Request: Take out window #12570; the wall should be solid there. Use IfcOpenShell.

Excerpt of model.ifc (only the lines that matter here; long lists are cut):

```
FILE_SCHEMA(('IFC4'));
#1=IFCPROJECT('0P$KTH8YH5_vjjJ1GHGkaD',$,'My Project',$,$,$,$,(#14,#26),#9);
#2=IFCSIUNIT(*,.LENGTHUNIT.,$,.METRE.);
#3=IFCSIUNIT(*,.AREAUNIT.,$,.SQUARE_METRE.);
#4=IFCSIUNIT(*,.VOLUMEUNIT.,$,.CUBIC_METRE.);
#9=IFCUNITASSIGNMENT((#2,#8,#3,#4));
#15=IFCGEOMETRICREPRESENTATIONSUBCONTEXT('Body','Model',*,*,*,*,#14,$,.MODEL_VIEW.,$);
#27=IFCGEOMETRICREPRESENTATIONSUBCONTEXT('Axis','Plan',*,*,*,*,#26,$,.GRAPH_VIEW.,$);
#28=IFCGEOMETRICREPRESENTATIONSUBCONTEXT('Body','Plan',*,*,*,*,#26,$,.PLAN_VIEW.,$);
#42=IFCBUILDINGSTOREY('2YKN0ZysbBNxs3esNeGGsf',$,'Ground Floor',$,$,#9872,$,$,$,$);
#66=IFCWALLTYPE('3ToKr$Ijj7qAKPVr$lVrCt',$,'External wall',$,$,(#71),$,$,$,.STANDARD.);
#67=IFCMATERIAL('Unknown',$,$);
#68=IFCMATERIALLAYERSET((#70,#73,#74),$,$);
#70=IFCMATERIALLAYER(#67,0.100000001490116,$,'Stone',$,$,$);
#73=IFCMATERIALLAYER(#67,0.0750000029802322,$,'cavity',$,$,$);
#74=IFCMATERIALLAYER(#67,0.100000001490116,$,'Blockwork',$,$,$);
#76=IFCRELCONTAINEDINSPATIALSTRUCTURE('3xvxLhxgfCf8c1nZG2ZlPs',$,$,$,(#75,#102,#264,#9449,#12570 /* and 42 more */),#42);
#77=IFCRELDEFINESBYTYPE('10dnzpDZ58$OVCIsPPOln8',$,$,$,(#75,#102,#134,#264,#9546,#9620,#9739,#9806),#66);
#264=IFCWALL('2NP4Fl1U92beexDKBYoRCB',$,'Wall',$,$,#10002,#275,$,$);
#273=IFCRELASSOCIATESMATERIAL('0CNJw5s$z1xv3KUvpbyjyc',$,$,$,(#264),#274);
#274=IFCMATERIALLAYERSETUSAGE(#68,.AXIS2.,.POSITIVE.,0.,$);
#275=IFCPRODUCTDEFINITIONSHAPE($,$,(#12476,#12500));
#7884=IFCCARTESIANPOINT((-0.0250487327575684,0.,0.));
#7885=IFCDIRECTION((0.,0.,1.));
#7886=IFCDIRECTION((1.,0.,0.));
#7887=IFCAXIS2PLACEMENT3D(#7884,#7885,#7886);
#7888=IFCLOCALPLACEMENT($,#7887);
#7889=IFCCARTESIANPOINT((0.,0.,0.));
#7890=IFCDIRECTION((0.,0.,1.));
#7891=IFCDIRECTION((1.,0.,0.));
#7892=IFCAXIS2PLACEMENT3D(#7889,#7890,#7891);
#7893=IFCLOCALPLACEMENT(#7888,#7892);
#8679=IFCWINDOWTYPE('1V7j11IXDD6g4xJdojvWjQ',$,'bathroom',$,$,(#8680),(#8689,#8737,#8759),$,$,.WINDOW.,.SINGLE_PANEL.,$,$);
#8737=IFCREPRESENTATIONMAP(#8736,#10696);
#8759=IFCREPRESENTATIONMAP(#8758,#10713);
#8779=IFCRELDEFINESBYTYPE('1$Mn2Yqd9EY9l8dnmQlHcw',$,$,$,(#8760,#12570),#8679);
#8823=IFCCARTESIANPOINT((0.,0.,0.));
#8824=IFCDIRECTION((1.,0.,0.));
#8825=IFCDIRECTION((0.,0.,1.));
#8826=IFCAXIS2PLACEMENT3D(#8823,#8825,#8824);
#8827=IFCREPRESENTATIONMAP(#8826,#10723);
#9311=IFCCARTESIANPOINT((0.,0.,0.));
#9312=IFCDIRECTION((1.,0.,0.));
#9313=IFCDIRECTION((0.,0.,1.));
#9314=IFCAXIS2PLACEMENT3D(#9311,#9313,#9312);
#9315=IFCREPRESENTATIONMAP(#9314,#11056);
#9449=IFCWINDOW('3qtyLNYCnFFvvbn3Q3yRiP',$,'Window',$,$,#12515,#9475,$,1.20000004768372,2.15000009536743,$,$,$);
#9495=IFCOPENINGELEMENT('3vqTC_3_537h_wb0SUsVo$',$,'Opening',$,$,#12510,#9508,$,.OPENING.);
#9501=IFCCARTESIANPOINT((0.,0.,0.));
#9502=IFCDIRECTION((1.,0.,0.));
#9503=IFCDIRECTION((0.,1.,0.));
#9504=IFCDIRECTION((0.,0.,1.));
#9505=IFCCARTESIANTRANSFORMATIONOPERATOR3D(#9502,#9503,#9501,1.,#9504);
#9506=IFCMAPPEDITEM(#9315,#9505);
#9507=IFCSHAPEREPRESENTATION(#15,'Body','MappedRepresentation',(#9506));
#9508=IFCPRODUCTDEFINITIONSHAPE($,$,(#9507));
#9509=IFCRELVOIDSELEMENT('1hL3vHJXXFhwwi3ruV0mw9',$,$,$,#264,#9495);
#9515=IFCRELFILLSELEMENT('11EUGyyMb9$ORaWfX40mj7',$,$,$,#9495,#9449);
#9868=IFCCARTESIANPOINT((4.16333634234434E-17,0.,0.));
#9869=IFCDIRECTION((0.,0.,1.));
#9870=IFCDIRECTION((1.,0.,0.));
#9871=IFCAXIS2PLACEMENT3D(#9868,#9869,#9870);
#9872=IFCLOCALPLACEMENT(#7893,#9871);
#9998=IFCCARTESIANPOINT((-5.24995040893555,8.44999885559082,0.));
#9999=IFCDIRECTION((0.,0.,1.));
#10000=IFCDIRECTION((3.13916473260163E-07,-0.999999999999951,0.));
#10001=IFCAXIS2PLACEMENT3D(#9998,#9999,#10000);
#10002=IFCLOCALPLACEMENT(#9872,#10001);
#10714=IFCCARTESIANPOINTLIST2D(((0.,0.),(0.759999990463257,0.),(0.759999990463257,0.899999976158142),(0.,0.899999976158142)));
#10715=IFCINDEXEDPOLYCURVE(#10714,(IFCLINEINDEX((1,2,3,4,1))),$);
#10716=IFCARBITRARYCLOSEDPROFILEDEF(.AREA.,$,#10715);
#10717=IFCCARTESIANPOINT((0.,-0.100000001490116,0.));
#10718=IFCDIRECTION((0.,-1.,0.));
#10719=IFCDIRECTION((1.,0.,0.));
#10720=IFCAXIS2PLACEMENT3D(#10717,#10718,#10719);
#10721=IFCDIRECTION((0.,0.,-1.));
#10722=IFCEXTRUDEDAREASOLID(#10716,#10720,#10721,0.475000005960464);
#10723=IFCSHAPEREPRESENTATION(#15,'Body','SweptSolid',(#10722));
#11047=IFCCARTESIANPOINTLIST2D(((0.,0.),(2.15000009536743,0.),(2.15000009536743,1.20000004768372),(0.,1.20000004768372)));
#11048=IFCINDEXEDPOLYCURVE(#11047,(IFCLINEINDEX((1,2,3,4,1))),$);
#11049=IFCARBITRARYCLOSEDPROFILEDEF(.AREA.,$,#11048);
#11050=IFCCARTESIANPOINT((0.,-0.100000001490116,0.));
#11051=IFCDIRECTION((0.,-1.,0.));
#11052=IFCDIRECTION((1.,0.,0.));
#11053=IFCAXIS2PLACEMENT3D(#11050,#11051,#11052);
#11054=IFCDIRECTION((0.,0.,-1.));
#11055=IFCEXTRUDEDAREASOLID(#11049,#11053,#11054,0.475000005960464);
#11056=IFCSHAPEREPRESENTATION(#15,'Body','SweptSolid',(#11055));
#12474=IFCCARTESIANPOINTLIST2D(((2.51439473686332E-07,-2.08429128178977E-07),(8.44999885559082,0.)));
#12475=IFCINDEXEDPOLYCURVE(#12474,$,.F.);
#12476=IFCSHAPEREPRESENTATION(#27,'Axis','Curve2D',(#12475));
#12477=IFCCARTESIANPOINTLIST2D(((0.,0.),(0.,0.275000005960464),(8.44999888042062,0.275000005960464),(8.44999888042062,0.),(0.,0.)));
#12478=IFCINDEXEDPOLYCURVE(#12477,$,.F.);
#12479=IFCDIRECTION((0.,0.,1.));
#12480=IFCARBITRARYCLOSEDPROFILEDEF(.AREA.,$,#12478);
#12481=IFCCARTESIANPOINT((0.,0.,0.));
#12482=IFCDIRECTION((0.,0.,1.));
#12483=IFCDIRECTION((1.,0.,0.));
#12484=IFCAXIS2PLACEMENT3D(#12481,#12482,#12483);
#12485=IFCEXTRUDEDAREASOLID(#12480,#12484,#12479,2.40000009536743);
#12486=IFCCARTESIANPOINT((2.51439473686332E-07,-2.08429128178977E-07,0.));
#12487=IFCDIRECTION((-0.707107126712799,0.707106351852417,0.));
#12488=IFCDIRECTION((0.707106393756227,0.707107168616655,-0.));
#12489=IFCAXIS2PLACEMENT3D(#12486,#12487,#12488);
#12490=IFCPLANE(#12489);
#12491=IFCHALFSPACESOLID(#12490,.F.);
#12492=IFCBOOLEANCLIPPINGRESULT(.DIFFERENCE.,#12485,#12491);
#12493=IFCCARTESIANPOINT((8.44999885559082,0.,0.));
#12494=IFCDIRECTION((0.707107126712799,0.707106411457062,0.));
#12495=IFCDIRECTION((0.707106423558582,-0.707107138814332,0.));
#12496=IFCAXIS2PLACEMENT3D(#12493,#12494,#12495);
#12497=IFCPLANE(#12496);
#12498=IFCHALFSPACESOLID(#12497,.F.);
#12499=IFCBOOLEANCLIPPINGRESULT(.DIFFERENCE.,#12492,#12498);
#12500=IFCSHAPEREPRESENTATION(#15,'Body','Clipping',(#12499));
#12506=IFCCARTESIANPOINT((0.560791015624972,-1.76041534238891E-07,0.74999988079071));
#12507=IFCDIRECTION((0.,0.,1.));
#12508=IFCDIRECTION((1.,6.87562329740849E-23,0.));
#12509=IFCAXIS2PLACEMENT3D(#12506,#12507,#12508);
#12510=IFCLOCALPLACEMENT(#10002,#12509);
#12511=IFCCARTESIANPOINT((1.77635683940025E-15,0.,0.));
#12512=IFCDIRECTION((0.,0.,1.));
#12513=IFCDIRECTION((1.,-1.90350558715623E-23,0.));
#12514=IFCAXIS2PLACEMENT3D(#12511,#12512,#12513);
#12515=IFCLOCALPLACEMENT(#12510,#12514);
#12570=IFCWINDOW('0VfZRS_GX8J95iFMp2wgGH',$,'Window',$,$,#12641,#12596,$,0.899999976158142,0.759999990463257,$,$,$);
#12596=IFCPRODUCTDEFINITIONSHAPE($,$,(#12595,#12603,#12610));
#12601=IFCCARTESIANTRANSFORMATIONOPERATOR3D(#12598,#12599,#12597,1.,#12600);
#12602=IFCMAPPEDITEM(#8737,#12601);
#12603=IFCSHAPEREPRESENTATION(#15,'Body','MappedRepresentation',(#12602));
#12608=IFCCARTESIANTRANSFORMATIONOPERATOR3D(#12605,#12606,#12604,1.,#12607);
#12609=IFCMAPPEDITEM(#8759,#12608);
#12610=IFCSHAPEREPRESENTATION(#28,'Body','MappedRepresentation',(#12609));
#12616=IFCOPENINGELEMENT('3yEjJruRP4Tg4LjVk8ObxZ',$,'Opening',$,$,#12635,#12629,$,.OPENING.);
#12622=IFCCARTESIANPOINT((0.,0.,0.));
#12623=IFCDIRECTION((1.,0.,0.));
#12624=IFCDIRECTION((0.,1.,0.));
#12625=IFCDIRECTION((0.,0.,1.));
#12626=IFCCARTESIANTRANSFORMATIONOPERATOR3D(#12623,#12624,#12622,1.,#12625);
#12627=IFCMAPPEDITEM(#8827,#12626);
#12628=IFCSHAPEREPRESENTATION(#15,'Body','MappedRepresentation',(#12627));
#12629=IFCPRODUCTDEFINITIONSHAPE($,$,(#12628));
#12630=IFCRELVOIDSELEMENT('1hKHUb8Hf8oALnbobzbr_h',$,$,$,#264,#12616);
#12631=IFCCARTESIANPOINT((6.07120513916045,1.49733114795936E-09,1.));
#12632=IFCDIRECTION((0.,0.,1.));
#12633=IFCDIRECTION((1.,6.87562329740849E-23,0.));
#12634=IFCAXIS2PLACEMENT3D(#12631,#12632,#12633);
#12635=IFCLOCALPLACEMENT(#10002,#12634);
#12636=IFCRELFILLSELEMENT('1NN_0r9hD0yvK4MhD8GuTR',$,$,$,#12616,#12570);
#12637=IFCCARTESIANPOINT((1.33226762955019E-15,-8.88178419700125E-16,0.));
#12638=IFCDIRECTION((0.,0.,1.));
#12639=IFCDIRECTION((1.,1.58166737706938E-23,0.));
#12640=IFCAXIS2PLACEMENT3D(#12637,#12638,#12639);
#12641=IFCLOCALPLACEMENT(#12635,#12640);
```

```python
import ifcopenshell
import ifcopenshell.api.feature
import ifcopenshell.api.root
import ifcopenshell.geom
import ifcopenshell.util.shape

model = ifcopenshell.open("model.ifc")
settings = ifcopenshell.geom.settings()


def volume(element):
    """Net volume in cubic metres, openings subtracted."""
    shape = ifcopenshell.geom.create_shape(settings, element)
    return ifcopenshell.util.shape.get_volume(shape.geometry)


window = model.by_guid("0VfZRS_GX8J95iFMp2wgGH")
opening = window.FillsVoids[0].RelatingOpeningElement
wall = opening.VoidsElements[0].RelatingBuildingElement
before = volume(wall)

ifcopenshell.api.root.remove_product(model, product=window)
ifcopenshell.api.feature.remove_feature(model, feature=opening)

after = volume(wall)

print(f"wall volume {before:.3f} -> {after:.3f} m3")

model.write("model_rev.ifc")
```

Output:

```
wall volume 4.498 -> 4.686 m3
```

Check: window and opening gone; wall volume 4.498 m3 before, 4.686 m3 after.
